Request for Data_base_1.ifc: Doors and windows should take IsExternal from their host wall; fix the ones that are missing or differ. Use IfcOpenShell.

First a look at what the model holds.

```python
import ifcopenshell
import ifcopenshell.util.element

model = ifcopenshell.open("Data_base_1.ifc")
print(model.schema)
seen = {}
for e in model.by_type("IfcDoor") + model.by_type("IfcWindow"):
    if not e.FillsVoids:
        continue
    host = e.FillsVoids[0].RelatingOpeningElement.VoidsElements[0].RelatingBuildingElement
    own = ifcopenshell.util.element.get_pset(e, f"Pset_{e.is_a()[3:].removesuffix('StandardCase')}Common", "IsExternal")
    wall = ifcopenshell.util.element.get_pset(host, "Pset_WallCommon", "IsExternal")
    seen[e.is_a(), own, wall] = seen.get((e.is_a(), own, wall), 0) + 1
for (cls, own, wall), count in sorted(seen.items(), key=str):
    print(count, cls, "IsExternal:", own, "| host wall:", wall)
```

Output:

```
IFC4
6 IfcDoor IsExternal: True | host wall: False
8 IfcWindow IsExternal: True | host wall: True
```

```python
import ifcopenshell
import ifcopenshell.api.pset
import ifcopenshell.util.element

model = ifcopenshell.open("Data_base_1.ifc")

count = 0
for ifc_class, pset_name in (("IfcDoor", "Pset_DoorCommon"), ("IfcWindow", "Pset_WindowCommon")):
    for e in model.by_type(ifc_class):
        if not e.FillsVoids:
            continue
        host = e.FillsVoids[0].RelatingOpeningElement.VoidsElements[0].RelatingBuildingElement
        external = ifcopenshell.util.element.get_pset(host, "Pset_WallCommon", "IsExternal")
        if external is None or ifcopenshell.util.element.get_pset(e, pset_name, "IsExternal") == external:
            continue
        pset = ifcopenshell.api.pset.add_pset(model, product=e, name=pset_name)
        ifcopenshell.api.pset.edit_pset(model, pset=pset, properties={"IsExternal": external})
        count += 1

print(count, "updated")

model.write("Data_base_1_updated.ifc")
```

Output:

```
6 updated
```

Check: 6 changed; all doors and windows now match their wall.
